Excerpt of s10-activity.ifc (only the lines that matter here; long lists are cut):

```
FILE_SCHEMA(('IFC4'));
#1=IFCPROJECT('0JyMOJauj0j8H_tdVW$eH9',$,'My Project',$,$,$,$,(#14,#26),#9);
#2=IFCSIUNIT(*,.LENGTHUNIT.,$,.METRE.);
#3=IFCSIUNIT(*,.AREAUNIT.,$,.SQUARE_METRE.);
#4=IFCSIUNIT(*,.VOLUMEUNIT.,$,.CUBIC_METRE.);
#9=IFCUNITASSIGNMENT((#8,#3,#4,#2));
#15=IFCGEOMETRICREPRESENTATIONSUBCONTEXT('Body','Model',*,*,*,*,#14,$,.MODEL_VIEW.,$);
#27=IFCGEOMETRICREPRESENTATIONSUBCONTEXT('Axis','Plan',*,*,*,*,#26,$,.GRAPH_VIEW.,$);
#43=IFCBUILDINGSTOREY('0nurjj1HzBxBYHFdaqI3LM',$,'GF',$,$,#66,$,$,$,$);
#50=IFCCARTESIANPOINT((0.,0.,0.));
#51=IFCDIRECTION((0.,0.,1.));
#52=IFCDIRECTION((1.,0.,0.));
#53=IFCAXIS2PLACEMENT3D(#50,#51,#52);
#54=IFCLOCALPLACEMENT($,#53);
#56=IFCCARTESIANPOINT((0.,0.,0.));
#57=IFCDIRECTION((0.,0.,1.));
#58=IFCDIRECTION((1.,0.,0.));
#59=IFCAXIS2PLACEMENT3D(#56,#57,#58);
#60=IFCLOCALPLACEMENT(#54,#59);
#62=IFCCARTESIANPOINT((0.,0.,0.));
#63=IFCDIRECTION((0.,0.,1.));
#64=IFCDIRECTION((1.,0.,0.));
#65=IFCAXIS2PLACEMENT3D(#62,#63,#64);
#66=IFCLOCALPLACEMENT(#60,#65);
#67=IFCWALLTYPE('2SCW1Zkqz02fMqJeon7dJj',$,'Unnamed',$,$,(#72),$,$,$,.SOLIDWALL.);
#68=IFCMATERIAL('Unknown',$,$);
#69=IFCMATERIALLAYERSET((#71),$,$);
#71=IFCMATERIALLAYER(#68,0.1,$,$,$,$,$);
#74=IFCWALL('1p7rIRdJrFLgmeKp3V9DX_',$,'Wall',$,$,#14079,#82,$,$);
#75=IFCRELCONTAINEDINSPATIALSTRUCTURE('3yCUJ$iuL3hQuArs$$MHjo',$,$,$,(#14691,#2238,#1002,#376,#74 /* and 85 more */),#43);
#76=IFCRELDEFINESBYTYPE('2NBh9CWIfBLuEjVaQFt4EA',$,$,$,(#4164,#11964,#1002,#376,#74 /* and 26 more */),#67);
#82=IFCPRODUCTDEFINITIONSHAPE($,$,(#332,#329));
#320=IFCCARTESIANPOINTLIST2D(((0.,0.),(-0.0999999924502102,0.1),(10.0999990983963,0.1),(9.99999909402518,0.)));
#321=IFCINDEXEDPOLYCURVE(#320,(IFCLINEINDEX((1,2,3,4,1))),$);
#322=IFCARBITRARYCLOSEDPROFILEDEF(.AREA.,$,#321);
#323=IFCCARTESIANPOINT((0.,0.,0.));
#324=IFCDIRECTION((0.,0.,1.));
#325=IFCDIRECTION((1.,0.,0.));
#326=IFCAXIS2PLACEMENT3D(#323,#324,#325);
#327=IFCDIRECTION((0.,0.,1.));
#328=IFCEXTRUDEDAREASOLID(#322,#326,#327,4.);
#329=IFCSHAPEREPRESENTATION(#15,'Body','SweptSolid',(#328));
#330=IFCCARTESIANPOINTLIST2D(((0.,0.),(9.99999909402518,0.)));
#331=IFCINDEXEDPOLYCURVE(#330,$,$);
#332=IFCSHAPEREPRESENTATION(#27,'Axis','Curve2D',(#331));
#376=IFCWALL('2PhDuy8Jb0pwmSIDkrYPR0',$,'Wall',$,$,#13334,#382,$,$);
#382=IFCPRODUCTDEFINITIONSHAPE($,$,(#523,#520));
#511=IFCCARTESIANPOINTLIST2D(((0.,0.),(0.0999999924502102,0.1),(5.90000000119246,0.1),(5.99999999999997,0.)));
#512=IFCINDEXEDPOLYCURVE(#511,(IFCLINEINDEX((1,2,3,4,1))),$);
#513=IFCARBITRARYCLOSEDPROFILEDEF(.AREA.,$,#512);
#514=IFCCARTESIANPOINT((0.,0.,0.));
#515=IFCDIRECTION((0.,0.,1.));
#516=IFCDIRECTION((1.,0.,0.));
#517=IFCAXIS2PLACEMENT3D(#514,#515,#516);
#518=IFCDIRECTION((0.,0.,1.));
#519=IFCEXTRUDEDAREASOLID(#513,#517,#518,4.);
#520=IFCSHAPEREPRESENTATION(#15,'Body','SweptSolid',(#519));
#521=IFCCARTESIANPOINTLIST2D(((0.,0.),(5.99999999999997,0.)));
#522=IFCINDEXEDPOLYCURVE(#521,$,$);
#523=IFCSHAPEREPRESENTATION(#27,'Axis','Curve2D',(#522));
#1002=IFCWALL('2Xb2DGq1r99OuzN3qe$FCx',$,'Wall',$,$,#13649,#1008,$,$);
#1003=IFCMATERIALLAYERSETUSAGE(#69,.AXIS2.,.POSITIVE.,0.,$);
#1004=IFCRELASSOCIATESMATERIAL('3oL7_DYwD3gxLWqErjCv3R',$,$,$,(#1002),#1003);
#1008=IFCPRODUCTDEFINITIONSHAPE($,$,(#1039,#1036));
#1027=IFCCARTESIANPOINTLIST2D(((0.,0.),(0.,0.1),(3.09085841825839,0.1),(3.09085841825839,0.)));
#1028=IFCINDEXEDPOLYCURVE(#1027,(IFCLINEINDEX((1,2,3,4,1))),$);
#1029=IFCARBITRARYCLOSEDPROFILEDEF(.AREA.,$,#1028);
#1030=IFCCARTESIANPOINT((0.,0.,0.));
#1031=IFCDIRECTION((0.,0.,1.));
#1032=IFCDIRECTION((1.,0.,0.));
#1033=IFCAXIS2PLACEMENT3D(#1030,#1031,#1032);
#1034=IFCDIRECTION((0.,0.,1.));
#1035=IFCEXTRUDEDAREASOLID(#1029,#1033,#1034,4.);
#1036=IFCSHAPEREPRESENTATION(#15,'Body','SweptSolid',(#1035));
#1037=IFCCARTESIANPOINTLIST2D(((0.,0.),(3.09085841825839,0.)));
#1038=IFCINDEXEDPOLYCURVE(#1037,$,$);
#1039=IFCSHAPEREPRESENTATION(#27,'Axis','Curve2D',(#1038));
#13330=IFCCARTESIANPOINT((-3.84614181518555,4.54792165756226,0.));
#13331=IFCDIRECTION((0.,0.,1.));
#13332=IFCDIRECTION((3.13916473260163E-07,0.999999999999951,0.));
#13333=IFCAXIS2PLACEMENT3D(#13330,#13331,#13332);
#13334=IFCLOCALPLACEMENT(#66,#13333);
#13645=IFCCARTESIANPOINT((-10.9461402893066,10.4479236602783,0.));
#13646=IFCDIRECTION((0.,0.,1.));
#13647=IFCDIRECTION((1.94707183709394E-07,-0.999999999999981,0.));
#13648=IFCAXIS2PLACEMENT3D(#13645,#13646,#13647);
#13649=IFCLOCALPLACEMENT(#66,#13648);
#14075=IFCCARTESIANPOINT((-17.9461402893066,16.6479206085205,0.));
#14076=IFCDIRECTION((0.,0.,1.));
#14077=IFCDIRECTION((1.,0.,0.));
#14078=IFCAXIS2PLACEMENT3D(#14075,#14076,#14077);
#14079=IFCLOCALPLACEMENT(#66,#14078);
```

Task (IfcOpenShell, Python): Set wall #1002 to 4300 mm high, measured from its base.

```python
import ifcopenshell
import ifcopenshell.geom
import ifcopenshell.util.representation
import ifcopenshell.util.shape
import ifcopenshell.util.unit

model = ifcopenshell.open("s10-activity.ifc")
unit_scale = ifcopenshell.util.unit.calculate_unit_scale(model)
settings = ifcopenshell.geom.settings()


def volume(element):
    """Net volume in cubic metres, openings subtracted."""
    shape = ifcopenshell.geom.create_shape(settings, element)
    return ifcopenshell.util.shape.get_volume(shape.geometry)


wall = model.by_guid("2Xb2DGq1r99OuzN3qe$FCx")
before = volume(wall)

body = ifcopenshell.util.representation.get_representation(wall, "Model", "Body")
solid = body.Items[0]
old_height = solid.Depth
solid.Depth = 4.3 / unit_scale
after = volume(wall)

print(f"height {old_height:g} -> {solid.Depth:g}, volume {before:.3f} -> {after:.3f} m3")

model.write("s10-activity_v2.ifc")
```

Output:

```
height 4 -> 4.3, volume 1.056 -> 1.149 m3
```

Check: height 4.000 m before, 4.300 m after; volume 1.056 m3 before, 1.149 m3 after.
